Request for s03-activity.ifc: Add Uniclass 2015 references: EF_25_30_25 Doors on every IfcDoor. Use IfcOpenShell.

First a look at what the model holds.

```python
import ifcopenshell

model = ifcopenshell.open("s03-activity.ifc")
print(model.schema)
print("classifications:", [c.Name for c in model.by_type("IfcClassification")])
for ifc_class in ("IfcDoor", "IfcRoof", "IfcStair", "IfcWall", "IfcWindow"):
    print(ifc_class, len(model.by_type(ifc_class)))
```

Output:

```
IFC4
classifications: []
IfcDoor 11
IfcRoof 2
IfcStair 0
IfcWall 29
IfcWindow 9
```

```python
import ifcopenshell
import ifcopenshell.api.classification

model = ifcopenshell.open("s03-activity.ifc")

system = ifcopenshell.api.classification.add_classification(model, classification="Uniclass 2015")

codes = {
    "IfcDoor": ("EF_25_30_25", "Doors"),
}
for ifc_class, (code, name) in codes.items():
    products = model.by_type(ifc_class)
    ifcopenshell.api.classification.add_reference(
        model, products=products, classification=system, identification=code, name=name
    )
    print(code, len(products))

model.write("s03-activity-out.ifc")
```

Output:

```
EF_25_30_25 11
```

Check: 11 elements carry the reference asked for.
